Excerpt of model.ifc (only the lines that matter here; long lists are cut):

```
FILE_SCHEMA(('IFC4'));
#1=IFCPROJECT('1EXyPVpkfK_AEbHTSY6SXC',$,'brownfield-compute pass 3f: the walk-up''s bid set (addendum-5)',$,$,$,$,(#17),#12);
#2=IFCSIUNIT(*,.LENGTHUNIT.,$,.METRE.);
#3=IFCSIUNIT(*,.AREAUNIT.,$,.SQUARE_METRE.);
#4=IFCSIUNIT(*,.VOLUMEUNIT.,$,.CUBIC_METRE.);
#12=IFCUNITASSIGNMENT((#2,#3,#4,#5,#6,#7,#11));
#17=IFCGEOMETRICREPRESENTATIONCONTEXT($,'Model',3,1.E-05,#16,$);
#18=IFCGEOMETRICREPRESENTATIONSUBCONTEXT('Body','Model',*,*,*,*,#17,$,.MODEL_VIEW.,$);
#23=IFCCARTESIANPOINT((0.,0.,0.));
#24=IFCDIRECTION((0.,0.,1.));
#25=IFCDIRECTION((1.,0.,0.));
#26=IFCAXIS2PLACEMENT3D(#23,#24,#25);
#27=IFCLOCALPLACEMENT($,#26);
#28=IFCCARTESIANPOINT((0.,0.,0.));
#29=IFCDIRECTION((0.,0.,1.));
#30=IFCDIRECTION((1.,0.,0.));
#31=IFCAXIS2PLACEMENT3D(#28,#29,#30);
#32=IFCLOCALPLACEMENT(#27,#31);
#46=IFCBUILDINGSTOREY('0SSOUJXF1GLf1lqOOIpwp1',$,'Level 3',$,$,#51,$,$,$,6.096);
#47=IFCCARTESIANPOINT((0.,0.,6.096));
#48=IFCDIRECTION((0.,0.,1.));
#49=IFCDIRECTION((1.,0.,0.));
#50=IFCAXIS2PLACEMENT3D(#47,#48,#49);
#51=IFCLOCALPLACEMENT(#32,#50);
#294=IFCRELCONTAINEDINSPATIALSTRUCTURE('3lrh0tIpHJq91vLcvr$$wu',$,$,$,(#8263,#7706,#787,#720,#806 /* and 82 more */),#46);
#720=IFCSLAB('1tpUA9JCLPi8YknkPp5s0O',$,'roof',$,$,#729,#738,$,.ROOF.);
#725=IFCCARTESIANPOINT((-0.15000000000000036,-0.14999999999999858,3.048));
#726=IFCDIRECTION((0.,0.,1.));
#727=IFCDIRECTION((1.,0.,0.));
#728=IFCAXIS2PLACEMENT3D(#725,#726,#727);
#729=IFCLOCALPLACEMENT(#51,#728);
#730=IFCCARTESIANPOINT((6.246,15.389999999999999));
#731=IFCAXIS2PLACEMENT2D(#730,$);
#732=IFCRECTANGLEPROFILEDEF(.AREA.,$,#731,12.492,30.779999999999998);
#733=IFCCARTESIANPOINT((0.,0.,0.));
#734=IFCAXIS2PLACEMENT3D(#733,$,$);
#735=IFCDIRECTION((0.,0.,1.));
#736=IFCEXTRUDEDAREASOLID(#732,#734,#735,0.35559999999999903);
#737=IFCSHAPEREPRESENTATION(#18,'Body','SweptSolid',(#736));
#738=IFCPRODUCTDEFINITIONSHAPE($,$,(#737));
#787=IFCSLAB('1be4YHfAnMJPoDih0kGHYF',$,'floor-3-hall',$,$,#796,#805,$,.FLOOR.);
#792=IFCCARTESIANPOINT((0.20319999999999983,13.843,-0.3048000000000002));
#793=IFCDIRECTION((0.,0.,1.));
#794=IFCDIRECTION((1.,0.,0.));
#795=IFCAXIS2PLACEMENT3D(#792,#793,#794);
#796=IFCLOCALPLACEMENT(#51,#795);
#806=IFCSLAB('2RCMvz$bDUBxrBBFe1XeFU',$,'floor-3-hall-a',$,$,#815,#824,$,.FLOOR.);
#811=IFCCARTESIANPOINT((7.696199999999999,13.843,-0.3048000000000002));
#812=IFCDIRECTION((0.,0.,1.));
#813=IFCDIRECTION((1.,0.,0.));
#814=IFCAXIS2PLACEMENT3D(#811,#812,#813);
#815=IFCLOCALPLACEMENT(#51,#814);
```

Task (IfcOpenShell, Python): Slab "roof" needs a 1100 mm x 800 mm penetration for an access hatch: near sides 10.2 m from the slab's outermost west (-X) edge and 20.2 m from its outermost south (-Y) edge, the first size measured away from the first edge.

```python
import numpy as np
import ifcopenshell
import ifcopenshell.api.feature
import ifcopenshell.api.geometry
import ifcopenshell.api.root
import ifcopenshell.geom
import ifcopenshell.util.placement
import ifcopenshell.util.representation
import ifcopenshell.util.shape
import ifcopenshell.util.unit

model = ifcopenshell.open("model.ifc")
unit_scale = ifcopenshell.util.unit.calculate_unit_scale(model)
settings = ifcopenshell.geom.settings()


def volume(element):
    """Net volume in cubic metres, openings subtracted."""
    shape = ifcopenshell.geom.create_shape(settings, element)
    return ifcopenshell.util.shape.get_volume(shape.geometry)


slab = model.by_guid("1tpUA9JCLPi8YknkPp5s0O")
before = volume(slab)

# Extent in the slab's own axes, in metres. The edges named are its -X and -Y sides.
slab_shape = ifcopenshell.geom.create_shape(settings, slab)
vertices = ifcopenshell.util.shape.get_vertices(slab_shape.geometry)
x_min, y_min, bottom = vertices.min(axis=0)
top = vertices[:, 2].max()

opening = ifcopenshell.api.root.create_entity(model, ifc_class="IfcOpeningElement", name="Access hatch opening", predefined_type="OPENING")
context = ifcopenshell.util.representation.get_context(model, "Model", "Body", "MODEL_VIEW")
width, depth = 1.1, 0.8
outline = [(0.0, 0.0), (width, 0.0), (width, depth), (0.0, depth), (0.0, 0.0)]
# Overshoot both faces by 50 mm so the cut is clean.
shape = ifcopenshell.api.geometry.add_slab_representation(
    model, context=context, depth=top - bottom + 0.1, polyline=outline
)
ifcopenshell.api.geometry.assign_representation(model, product=opening, representation=shape)

matrix = ifcopenshell.util.placement.get_local_placement(slab.ObjectPlacement)
matrix[:, 3] = matrix @ np.append(np.array([x_min + 10.2, y_min + 20.2, bottom - 0.05]) / unit_scale, 1.0)
ifcopenshell.api.geometry.edit_object_placement(model, product=opening, matrix=matrix, is_si=False)
ifcopenshell.api.feature.add_feature(model, feature=opening, element=slab)

after = volume(slab)

print(f"slab volume {before:.3f} -> {after:.3f} m3")

model.write("model_edited.ifc")
```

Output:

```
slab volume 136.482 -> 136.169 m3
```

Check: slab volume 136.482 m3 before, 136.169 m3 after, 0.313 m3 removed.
